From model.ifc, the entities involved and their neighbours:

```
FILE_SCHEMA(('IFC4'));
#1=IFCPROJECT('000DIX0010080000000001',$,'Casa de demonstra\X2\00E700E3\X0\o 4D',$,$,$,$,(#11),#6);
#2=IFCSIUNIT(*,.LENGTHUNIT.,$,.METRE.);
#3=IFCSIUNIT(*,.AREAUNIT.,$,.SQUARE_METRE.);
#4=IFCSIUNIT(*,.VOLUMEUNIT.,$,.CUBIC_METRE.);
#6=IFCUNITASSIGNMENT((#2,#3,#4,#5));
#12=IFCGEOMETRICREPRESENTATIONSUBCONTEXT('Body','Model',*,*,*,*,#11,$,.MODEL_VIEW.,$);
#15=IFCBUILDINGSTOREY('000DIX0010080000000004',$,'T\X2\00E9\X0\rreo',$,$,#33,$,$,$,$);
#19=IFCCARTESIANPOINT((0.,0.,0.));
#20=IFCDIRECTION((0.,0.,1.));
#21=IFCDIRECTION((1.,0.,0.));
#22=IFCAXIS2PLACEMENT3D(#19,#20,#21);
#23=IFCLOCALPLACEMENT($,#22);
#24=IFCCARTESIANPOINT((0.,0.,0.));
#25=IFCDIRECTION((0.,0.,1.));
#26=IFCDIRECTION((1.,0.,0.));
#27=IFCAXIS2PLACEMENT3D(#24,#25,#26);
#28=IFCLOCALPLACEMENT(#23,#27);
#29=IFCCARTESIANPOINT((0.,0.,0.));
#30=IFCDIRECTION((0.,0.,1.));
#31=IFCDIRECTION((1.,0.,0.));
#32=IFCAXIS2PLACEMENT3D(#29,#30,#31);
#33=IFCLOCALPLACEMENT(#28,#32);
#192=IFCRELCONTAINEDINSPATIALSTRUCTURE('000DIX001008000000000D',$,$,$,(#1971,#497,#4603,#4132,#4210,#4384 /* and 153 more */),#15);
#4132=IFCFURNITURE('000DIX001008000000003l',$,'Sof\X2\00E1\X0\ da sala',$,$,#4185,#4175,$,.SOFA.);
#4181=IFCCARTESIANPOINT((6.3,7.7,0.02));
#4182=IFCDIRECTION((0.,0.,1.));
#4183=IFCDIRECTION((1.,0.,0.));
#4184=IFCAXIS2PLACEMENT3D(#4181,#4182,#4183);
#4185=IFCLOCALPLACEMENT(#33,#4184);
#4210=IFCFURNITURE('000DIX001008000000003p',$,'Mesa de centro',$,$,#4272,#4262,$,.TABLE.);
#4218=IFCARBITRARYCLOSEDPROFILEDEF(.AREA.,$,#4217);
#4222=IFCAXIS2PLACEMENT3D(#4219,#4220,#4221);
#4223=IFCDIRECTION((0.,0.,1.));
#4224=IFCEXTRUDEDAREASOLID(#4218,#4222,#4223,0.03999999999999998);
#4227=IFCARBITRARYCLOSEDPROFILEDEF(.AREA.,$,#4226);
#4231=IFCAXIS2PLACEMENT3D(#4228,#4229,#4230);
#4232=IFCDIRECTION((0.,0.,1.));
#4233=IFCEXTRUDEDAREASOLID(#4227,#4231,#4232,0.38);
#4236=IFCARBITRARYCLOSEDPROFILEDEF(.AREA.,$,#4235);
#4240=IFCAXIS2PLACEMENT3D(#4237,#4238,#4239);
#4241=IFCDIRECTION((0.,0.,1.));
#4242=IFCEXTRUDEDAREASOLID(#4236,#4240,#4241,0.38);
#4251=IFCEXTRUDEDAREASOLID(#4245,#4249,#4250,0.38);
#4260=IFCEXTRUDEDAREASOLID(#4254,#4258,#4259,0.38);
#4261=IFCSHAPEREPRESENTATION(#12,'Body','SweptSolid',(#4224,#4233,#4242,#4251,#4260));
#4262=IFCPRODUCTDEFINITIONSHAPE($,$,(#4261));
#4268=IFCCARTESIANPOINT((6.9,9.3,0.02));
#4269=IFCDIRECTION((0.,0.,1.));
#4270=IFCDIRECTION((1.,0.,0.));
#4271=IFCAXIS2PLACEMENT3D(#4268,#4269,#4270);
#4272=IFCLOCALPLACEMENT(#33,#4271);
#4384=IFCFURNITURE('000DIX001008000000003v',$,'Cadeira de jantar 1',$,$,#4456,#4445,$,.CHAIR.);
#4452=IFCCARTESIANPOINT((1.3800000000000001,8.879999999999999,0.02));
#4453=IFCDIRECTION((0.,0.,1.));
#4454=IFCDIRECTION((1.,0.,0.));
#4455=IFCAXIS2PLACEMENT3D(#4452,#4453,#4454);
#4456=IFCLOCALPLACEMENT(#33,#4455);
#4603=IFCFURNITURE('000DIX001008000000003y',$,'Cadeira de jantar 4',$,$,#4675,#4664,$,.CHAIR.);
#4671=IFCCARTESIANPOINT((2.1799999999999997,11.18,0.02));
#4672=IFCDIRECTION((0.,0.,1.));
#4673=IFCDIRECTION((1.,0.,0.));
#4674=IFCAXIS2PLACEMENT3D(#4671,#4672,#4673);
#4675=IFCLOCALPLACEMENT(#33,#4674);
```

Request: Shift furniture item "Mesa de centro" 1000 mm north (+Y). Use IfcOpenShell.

```python
import ifcopenshell
import ifcopenshell.api.geometry
import ifcopenshell.util.placement

model = ifcopenshell.open("model.ifc")

item = model.by_guid("000DIX001008000000003p")
matrix = ifcopenshell.util.placement.get_local_placement(item.ObjectPlacement)
matrix[1, 3] += 1.0
ifcopenshell.api.geometry.edit_object_placement(model, product=item, matrix=matrix, is_si=False)

print(ifcopenshell.util.placement.get_local_placement(item.ObjectPlacement).round(3) + 0.0)

model.write("model-out.ifc")
```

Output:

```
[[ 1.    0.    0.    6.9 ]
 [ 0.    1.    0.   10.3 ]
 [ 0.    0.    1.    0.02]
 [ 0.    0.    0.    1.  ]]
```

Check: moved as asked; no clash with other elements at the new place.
